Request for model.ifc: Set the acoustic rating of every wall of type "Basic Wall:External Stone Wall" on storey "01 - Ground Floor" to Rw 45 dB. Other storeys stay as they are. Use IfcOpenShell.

First a look at what the model holds.

```python
import ifcopenshell
import ifcopenshell.util.element

model = ifcopenshell.open("model.ifc")
print(model.schema)
storey = next(s for s in model.by_type("IfcBuildingStorey") if s.Name == "01 - Ground Floor")
walls = [e for e in ifcopenshell.util.element.get_decomposition(storey) if e.is_a("IfcWall")]
seen = {}
for e in walls:
    element_type = ifcopenshell.util.element.get_type(e)
    key = (element_type.Name if element_type != e and element_type else None, ifcopenshell.util.element.get_pset(e, "Pset_WallCommon", "AcousticRating"))
    seen[key] = seen.get(key, 0) + 1
for (name, value), count in sorted(seen.items(), key=str):
    print(count, "x", name, "|", value)
```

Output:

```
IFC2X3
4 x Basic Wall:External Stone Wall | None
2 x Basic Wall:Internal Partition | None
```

```python
import ifcopenshell
import ifcopenshell.api.pset
import ifcopenshell.util.element

model = ifcopenshell.open("model.ifc")

storey = next(s for s in model.by_type("IfcBuildingStorey") if s.Name == "01 - Ground Floor")
walls = [e for e in ifcopenshell.util.element.get_decomposition(storey) if e.is_a("IfcWall")]

count = 0
for e in walls:
    element_type = ifcopenshell.util.element.get_type(e)
    if element_type in (None, e) or element_type.Name != "Basic Wall:External Stone Wall":
        continue
    # add_pset returns the element's existing set when there is one.
    pset = ifcopenshell.api.pset.add_pset(model, product=e, name="Pset_WallCommon")
    ifcopenshell.api.pset.edit_pset(model, pset=pset, properties={"AcousticRating": "Rw 45 dB"})
    count += 1

print(count, "walls updated")

model.write("model_edited.ifc")
```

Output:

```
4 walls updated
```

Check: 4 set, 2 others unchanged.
